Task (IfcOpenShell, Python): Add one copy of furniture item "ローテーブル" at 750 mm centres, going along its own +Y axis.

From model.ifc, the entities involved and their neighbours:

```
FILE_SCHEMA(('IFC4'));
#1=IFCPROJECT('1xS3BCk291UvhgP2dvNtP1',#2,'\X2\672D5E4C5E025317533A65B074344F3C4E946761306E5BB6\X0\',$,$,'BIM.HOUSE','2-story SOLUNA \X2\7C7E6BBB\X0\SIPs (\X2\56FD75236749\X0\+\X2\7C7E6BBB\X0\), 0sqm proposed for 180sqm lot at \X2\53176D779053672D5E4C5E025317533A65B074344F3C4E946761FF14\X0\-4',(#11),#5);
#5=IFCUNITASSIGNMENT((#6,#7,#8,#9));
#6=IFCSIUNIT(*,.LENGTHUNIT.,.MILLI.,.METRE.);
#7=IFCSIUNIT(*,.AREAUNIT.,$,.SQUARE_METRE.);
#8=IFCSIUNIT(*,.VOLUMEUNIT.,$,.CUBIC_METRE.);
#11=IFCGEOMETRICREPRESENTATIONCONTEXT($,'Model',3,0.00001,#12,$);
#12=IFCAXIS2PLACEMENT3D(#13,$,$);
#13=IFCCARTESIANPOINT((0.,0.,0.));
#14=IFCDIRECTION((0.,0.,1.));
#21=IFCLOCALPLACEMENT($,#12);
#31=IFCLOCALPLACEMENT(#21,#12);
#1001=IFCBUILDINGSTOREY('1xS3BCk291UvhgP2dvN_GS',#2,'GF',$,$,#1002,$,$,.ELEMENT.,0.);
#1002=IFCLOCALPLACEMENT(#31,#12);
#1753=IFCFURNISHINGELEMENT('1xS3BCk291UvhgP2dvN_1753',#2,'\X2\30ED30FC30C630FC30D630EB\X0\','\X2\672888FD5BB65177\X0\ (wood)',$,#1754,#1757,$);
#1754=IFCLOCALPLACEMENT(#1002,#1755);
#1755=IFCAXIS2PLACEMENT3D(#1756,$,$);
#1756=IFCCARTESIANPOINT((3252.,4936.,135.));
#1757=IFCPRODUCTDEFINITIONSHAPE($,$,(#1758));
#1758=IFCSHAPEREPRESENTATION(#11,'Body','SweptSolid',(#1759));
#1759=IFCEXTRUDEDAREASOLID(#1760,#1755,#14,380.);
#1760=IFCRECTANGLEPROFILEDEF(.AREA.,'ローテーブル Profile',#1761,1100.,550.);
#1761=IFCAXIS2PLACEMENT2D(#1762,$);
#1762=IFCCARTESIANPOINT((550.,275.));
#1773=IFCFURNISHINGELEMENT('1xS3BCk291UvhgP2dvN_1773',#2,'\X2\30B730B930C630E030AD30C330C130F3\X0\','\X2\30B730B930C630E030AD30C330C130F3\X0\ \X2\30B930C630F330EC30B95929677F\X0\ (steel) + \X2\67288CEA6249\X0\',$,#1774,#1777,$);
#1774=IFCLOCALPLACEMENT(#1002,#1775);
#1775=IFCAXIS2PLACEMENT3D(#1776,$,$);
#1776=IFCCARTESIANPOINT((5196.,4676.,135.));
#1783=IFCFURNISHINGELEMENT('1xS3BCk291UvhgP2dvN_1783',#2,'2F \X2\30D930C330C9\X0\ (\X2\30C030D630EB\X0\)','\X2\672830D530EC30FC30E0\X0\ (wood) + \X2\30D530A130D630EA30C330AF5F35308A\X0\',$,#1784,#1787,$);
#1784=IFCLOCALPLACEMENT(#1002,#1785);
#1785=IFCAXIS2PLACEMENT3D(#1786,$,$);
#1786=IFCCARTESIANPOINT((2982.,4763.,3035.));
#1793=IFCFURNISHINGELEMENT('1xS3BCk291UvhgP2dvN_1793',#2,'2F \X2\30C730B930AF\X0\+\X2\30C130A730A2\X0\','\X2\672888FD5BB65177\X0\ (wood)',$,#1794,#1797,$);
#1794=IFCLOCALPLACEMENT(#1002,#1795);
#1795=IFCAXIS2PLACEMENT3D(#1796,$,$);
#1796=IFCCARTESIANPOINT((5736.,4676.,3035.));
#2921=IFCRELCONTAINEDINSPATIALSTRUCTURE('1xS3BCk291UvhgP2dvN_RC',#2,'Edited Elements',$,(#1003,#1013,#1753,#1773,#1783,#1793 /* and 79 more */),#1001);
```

```python
import ifcopenshell
import ifcopenshell.api.geometry
import ifcopenshell.api.root
import ifcopenshell.util.element
import ifcopenshell.util.placement

model = ifcopenshell.open("model.ifc")


def reuse_history(source, copy):
    """copy_class also copies each property set's owner history, people and application; keep the originals."""
    for rel in copy.IsDefinedBy:
        if rel.is_a("IfcRelDefinesByProperties") and (history := rel.RelatingPropertyDefinition.OwnerHistory):
            rel.RelatingPropertyDefinition.OwnerHistory = source.OwnerHistory
            ifcopenshell.util.element.remove_deep2(model, history)


source = model.by_guid("1xS3BCk291UvhgP2dvN_1753")
base = ifcopenshell.util.placement.get_local_placement(source.ObjectPlacement)
step = base[:3, 1] * 750.0

for i in range(1, 2):
    copy = ifcopenshell.api.root.copy_class(model, product=source)
    copy.Representation = ifcopenshell.util.element.copy_deep(
        model, source.Representation, exclude=["IfcGeometricRepresentationContext", "IfcRepresentationMap"]
    )
    reuse_history(source, copy)
    matrix = base.copy()
    matrix[:3, 3] += i * step
    print("added at", matrix[:3, 3].round(3) + 0.0)
    ifcopenshell.api.geometry.edit_object_placement(model, product=copy, matrix=matrix, is_si=False)

model.write("model_updated.ifc")
```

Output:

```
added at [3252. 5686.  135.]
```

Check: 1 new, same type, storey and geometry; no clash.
